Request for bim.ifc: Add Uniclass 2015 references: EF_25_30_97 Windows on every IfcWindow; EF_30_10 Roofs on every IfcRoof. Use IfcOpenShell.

First a look at what the model holds.

```python
import ifcopenshell

model = ifcopenshell.open("bim.ifc")
print(model.schema)
print("classifications:", [c.Name for c in model.by_type("IfcClassification")])
for ifc_class in ("IfcDoor", "IfcRoof", "IfcStair", "IfcWall", "IfcWindow"):
    print(ifc_class, len(model.by_type(ifc_class)))
```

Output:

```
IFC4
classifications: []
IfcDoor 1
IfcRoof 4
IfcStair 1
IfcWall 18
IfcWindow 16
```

```python
import ifcopenshell
import ifcopenshell.api.classification

model = ifcopenshell.open("bim.ifc")

system = ifcopenshell.api.classification.add_classification(model, classification="Uniclass 2015")

codes = {
    "IfcWindow": ("EF_25_30_97", "Windows"),
    "IfcRoof": ("EF_30_10", "Roofs"),
}
for ifc_class, (code, name) in codes.items():
    products = model.by_type(ifc_class)
    ifcopenshell.api.classification.add_reference(
        model, products=products, classification=system, identification=code, name=name
    )
    print(code, len(products))

model.write("bim-out.ifc")
```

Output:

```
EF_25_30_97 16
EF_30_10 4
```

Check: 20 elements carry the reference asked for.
